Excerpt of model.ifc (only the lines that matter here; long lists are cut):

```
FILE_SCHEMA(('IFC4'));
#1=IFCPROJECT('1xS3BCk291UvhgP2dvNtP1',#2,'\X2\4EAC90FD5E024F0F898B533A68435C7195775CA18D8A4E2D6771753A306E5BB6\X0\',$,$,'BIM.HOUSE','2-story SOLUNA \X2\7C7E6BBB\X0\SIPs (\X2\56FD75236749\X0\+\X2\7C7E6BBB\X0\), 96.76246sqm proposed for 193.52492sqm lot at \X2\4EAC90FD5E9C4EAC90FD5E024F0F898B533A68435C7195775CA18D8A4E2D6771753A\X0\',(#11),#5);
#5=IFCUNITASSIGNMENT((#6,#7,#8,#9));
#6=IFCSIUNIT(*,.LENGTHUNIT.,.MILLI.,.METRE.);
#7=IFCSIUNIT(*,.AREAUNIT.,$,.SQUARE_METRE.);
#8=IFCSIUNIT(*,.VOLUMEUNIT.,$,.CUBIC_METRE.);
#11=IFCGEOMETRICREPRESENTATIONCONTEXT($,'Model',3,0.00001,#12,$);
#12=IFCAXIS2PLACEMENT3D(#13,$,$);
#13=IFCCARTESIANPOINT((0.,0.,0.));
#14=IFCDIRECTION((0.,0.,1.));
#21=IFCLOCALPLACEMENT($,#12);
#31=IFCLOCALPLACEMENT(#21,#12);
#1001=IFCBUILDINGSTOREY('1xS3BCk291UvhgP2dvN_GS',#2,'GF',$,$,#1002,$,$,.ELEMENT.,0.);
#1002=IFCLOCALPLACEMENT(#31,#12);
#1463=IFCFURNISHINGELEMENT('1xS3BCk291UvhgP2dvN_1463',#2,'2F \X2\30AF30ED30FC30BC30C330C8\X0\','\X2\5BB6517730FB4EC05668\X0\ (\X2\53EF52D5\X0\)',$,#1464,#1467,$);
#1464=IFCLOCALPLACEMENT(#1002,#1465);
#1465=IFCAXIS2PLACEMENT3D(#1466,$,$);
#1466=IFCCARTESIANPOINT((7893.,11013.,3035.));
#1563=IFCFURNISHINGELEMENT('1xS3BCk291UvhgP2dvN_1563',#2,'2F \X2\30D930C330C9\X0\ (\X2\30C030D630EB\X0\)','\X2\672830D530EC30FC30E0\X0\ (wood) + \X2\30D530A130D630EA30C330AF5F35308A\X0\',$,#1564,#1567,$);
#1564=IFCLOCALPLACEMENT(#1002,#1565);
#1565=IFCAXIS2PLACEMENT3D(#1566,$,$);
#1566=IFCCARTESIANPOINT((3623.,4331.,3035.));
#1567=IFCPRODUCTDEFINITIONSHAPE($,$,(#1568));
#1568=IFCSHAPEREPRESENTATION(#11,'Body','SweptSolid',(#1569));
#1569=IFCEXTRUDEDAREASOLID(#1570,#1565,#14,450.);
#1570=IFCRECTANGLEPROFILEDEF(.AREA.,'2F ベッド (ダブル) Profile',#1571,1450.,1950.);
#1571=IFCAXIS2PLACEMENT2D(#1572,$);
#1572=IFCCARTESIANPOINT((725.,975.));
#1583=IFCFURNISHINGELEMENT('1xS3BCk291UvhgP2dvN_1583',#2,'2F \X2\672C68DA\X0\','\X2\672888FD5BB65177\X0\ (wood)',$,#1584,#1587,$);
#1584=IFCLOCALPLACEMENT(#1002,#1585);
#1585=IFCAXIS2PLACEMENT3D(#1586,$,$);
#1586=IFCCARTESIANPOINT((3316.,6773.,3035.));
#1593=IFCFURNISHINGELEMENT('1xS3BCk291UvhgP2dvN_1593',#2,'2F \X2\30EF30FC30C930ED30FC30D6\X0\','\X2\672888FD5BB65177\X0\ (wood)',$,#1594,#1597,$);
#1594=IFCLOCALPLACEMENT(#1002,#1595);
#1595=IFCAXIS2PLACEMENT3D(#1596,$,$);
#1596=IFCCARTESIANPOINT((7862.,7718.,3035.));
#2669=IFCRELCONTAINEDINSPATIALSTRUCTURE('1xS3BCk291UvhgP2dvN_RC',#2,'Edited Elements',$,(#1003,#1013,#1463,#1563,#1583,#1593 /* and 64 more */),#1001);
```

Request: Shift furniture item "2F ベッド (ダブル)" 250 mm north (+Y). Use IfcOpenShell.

```python
import ifcopenshell
import ifcopenshell.api.geometry
import ifcopenshell.util.placement
import ifcopenshell.util.unit

model = ifcopenshell.open("model.ifc")
unit_scale = ifcopenshell.util.unit.calculate_unit_scale(model)

item = model.by_id(1563)
matrix = ifcopenshell.util.placement.get_local_placement(item.ObjectPlacement)
matrix[1, 3] += 0.25 / unit_scale
ifcopenshell.api.geometry.edit_object_placement(model, product=item, matrix=matrix, is_si=False)

print(ifcopenshell.util.placement.get_local_placement(item.ObjectPlacement).round(3) + 0.0)

model.write("model-out.ifc")
```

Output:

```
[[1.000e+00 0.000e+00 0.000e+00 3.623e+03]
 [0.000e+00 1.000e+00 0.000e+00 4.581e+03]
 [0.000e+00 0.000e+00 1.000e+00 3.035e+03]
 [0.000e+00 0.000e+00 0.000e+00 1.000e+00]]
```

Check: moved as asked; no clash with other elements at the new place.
